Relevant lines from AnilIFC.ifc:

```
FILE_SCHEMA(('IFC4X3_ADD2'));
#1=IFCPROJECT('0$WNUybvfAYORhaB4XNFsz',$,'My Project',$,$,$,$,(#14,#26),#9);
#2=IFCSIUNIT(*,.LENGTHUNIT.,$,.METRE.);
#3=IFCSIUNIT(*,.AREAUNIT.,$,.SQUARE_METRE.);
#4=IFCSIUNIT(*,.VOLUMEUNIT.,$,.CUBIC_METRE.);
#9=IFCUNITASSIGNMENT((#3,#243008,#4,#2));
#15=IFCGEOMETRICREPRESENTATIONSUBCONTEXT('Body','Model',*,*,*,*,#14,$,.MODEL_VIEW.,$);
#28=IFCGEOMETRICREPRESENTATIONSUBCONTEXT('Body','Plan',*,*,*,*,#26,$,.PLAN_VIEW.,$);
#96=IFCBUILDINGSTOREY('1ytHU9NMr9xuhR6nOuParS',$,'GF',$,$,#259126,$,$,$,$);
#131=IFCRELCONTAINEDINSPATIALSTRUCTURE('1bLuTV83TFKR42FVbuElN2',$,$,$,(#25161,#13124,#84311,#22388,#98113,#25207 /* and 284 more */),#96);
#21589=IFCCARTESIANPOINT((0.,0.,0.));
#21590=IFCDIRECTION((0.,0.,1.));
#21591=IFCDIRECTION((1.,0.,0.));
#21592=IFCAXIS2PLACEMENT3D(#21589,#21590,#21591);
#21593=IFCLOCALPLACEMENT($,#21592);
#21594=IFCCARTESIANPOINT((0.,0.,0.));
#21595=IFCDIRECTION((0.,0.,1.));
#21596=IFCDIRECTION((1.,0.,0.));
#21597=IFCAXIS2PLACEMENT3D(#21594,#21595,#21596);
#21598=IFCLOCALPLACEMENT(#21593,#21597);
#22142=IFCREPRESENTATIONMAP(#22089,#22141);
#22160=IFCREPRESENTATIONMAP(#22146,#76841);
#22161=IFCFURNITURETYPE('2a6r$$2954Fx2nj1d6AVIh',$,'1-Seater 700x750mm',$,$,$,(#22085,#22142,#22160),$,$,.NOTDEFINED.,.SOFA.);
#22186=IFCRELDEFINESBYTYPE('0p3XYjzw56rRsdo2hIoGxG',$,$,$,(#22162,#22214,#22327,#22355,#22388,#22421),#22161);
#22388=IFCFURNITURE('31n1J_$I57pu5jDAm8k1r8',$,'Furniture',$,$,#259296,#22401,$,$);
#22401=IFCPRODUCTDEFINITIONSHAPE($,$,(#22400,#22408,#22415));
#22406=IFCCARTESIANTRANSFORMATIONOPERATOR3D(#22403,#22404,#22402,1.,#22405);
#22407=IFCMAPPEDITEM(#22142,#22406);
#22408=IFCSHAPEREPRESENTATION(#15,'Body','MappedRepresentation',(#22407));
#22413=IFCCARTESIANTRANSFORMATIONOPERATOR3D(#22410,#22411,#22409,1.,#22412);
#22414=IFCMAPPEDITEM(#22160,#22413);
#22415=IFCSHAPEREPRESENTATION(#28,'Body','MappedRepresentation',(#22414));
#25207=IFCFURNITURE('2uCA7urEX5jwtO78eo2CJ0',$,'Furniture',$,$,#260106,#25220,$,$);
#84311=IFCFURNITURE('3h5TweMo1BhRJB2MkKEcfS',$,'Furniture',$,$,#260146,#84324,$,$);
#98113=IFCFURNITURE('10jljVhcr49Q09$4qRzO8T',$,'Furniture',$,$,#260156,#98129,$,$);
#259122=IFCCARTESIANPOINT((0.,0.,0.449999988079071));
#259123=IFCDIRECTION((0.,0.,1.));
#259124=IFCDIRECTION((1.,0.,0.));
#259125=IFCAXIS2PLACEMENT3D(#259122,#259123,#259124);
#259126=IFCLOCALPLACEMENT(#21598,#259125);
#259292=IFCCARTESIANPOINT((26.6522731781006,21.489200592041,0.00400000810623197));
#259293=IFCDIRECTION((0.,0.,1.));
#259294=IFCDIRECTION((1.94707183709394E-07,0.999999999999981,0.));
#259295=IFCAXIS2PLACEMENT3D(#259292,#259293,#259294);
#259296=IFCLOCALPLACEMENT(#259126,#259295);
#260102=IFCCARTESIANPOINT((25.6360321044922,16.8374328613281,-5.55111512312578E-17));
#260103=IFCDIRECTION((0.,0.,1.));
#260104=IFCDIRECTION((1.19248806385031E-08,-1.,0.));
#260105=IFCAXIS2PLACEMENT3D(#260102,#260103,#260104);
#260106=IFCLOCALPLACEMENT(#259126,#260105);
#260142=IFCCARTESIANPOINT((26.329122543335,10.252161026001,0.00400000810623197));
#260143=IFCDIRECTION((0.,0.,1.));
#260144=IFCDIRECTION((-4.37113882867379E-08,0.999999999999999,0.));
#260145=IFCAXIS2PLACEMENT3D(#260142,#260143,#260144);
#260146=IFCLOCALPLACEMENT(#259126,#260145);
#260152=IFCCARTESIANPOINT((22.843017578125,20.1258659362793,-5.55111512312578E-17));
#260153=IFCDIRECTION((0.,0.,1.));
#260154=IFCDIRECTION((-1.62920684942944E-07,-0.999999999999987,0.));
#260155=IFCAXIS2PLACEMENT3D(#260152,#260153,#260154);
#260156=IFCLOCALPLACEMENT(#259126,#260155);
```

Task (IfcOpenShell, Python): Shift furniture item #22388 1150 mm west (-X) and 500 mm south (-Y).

```python
import ifcopenshell
import ifcopenshell.api.geometry
import ifcopenshell.util.placement
import ifcopenshell.util.unit

model = ifcopenshell.open("AnilIFC.ifc")
unit_scale = ifcopenshell.util.unit.calculate_unit_scale(model)

item = model.by_id(22388)
matrix = ifcopenshell.util.placement.get_local_placement(item.ObjectPlacement)
matrix[0, 3] -= 1.15 / unit_scale
matrix[1, 3] -= 0.5 / unit_scale
ifcopenshell.api.geometry.edit_object_placement(model, product=item, matrix=matrix, is_si=False)

print(ifcopenshell.util.placement.get_local_placement(item.ObjectPlacement).round(3) + 0.0)

model.write("AnilIFC_rev.ifc")
```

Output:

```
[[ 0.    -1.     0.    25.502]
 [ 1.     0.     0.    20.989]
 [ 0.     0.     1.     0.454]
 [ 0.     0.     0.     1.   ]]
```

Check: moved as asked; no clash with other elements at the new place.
